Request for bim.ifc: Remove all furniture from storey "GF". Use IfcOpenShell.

First a look at what the model holds.

```python
import ifcopenshell
import ifcopenshell.util.element

model = ifcopenshell.open("bim.ifc")
print(model.schema)
storey = next(s for s in model.by_type("IfcBuildingStorey") if s.Name == "GF")
furniture = [e for e in ifcopenshell.util.element.get_decomposition(storey) if e.is_a("IfcFurnishingElement")]
seen = {}
for e in furniture:
    element_type = ifcopenshell.util.element.get_type(e)
    name = element_type.Name if element_type not in (None, e) else None
    seen[name] = seen.get(name, 0) + 1
for name, count in sorted(seen.items(), key=str):
    print(count, "x", name)
```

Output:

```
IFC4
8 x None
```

```python
import ifcopenshell
import ifcopenshell.api.root
import ifcopenshell.util.element

model = ifcopenshell.open("bim.ifc")

storey = next(s for s in model.by_type("IfcBuildingStorey") if s.Name == "GF")
furniture = [e for e in ifcopenshell.util.element.get_decomposition(storey) if e.is_a("IfcFurnishingElement")]

for e in furniture:
    ifcopenshell.api.root.remove_product(model, product=e)
print(len(furniture), "removed")

model.write("bim_rev.ifc")
```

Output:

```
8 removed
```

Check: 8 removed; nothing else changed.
